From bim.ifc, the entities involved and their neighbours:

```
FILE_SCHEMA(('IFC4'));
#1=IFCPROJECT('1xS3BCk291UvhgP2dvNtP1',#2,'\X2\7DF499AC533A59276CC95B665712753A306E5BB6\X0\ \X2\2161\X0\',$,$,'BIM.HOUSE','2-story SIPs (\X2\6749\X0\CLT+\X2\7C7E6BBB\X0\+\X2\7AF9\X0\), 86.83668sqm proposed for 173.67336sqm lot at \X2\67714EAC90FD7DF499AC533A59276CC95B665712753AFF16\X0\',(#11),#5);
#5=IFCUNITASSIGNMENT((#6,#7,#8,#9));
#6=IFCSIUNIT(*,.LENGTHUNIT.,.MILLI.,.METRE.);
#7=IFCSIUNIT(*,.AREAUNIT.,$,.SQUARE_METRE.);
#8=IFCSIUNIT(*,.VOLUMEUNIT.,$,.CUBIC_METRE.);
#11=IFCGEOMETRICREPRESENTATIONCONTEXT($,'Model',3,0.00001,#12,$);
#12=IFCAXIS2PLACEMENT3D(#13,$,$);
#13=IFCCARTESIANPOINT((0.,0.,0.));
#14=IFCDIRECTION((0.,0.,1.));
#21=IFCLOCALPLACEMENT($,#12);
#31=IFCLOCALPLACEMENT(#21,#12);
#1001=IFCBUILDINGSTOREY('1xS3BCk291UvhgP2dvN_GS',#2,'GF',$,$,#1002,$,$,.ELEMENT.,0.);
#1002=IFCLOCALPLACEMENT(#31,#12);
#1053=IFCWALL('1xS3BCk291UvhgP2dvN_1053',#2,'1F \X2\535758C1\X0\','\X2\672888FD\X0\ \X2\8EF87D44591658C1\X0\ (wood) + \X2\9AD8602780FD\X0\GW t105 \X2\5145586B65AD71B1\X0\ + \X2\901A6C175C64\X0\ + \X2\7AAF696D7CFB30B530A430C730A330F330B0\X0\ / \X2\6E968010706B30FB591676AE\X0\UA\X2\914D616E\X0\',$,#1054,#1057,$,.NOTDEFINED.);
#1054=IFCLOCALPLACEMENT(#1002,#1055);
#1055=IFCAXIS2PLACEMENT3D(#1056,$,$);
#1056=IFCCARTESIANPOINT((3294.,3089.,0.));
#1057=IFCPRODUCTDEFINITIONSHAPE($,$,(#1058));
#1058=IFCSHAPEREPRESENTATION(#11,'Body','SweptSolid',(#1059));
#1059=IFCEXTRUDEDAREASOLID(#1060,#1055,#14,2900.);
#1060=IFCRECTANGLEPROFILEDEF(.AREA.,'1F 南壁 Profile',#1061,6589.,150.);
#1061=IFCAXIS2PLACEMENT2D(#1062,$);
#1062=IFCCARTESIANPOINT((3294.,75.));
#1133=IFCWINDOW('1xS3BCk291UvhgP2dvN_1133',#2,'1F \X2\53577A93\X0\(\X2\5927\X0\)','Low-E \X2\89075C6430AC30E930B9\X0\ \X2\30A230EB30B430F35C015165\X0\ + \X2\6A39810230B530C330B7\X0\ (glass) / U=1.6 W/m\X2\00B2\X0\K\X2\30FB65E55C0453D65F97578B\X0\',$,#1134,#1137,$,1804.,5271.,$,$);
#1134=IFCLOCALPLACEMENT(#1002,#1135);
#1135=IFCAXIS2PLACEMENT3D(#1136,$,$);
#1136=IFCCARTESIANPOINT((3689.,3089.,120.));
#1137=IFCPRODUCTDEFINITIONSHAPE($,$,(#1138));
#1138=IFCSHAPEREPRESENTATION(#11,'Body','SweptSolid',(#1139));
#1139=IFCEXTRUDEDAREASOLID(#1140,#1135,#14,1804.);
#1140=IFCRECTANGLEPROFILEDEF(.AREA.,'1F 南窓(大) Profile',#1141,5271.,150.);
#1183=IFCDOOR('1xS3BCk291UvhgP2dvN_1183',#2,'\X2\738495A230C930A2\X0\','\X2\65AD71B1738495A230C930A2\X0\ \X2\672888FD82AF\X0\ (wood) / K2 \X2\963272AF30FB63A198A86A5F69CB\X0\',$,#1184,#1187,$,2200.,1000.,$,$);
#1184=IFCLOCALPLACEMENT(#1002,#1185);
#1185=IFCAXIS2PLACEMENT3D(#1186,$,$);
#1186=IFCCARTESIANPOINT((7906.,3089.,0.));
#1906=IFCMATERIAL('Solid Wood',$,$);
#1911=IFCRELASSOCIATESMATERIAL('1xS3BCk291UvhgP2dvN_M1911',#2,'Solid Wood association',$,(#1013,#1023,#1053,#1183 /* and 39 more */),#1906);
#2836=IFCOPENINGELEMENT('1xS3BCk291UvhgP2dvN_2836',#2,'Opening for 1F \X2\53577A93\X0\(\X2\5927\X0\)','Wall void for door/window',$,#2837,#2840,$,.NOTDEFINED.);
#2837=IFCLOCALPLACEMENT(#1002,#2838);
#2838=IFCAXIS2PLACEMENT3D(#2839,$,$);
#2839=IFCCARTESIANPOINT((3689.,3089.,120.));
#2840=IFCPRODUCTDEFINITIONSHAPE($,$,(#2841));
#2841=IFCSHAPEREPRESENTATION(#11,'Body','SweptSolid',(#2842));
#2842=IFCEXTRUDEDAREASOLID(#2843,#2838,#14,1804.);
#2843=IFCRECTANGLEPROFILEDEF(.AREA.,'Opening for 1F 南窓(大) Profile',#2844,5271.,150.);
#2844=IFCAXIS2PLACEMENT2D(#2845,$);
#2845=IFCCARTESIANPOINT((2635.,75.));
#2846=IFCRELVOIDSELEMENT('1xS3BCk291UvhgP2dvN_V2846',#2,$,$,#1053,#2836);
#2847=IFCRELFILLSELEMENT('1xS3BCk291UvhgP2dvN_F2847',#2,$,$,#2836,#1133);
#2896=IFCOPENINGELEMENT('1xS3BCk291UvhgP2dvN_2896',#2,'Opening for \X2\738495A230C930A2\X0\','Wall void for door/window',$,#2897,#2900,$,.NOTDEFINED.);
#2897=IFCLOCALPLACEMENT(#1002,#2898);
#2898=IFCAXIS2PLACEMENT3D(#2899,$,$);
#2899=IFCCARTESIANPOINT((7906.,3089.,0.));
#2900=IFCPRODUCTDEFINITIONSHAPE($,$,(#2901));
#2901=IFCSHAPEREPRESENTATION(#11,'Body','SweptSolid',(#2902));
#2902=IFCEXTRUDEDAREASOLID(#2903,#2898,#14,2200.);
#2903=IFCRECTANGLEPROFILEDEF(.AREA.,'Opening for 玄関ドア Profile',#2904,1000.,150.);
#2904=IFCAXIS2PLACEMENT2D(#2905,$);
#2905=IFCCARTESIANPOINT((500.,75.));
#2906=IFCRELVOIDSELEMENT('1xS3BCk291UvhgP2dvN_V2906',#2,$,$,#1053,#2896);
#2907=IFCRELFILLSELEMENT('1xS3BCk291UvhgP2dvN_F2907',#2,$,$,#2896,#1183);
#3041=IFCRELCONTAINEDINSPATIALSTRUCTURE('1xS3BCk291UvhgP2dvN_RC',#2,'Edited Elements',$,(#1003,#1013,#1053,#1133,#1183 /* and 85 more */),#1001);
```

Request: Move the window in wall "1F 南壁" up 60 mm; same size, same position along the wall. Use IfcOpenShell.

```python
import numpy as np
import ifcopenshell
import ifcopenshell.api.geometry
import ifcopenshell.util.placement
import ifcopenshell.util.unit

model = ifcopenshell.open("bim.ifc")
unit_scale = ifcopenshell.util.unit.calculate_unit_scale(model)

window = model.by_guid("1xS3BCk291UvhgP2dvN_1133")
opening = window.FillsVoids[0].RelatingOpeningElement
dz = 0.06 / unit_scale

shift = np.array([0.0, 0.0, dz])
# The window is not placed relative to its opening, so move both.
for product in (opening, window):
    matrix = ifcopenshell.util.placement.get_local_placement(product.ObjectPlacement)
    matrix[:3, 3] += shift
    ifcopenshell.api.geometry.edit_object_placement(model, product=product, matrix=matrix, is_si=False)

print(f"moved by {dz * unit_scale:+.3f} m")

model.write("bim-out.ifc")
```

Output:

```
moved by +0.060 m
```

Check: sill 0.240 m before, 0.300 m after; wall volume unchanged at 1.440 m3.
